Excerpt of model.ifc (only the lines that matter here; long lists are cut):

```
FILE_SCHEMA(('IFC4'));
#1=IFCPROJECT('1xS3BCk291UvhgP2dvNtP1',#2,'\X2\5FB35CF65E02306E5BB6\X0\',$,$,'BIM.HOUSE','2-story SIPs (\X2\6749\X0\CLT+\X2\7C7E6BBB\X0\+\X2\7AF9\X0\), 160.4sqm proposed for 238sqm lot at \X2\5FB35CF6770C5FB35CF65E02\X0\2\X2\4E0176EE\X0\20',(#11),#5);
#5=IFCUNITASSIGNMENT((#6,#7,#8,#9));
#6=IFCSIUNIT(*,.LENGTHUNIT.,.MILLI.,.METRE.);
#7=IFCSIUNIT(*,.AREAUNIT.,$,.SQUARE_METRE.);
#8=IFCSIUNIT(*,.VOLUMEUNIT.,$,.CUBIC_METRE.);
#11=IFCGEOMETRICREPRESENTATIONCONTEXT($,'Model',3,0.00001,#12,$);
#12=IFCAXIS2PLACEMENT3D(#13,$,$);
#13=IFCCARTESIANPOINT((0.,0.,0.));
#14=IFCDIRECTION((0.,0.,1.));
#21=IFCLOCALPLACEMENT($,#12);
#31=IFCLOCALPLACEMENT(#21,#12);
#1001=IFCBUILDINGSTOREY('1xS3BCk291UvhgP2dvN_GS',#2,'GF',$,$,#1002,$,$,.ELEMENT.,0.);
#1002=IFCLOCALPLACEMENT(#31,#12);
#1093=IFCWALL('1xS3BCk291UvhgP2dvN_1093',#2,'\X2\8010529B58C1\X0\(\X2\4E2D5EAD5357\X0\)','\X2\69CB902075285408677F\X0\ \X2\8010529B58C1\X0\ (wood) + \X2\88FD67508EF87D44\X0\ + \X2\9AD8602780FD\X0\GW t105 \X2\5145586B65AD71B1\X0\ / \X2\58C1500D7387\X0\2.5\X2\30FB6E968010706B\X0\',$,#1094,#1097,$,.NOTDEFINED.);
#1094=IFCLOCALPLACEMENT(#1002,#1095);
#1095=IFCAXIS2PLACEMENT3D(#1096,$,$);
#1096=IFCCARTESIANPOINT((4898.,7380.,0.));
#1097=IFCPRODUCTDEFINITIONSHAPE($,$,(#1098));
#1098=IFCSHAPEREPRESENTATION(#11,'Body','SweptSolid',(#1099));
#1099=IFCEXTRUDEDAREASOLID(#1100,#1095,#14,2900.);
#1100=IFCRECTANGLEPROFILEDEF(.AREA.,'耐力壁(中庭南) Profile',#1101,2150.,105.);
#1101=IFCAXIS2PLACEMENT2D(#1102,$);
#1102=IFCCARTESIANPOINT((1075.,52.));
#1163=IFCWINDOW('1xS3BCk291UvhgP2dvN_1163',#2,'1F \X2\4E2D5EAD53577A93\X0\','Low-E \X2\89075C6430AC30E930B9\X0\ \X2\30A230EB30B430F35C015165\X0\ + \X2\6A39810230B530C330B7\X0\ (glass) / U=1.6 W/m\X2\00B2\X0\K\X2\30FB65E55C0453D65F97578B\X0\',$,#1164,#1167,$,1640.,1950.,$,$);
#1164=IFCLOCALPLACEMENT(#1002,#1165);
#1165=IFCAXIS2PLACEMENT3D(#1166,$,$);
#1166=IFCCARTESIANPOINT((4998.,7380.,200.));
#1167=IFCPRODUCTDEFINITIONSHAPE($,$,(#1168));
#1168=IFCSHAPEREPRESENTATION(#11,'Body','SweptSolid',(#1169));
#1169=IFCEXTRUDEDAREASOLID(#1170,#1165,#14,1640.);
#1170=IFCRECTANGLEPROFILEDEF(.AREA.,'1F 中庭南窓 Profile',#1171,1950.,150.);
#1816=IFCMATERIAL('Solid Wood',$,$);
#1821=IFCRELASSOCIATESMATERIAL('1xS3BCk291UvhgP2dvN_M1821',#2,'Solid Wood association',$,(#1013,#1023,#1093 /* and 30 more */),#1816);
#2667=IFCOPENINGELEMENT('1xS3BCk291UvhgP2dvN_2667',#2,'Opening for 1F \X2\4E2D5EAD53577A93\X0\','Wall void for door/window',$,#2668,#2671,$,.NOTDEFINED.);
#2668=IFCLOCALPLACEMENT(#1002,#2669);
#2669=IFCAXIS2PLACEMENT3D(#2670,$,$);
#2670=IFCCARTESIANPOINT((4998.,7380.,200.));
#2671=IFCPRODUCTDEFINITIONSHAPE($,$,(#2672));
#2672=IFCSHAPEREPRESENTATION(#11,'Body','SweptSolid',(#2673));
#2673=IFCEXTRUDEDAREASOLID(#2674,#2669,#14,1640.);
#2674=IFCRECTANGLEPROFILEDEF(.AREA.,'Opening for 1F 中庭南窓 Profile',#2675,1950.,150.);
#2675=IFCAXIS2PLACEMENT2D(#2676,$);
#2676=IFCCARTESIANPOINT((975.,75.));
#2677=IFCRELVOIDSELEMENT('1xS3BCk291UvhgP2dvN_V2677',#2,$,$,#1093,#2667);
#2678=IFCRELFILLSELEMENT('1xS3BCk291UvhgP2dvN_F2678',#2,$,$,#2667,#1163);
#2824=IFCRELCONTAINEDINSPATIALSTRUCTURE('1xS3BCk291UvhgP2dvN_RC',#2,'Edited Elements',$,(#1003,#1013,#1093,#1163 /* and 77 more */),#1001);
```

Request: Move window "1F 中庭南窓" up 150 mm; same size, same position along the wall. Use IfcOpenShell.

```python
import numpy as np
import ifcopenshell
import ifcopenshell.api.geometry
import ifcopenshell.util.placement
import ifcopenshell.util.unit

model = ifcopenshell.open("model.ifc")
unit_scale = ifcopenshell.util.unit.calculate_unit_scale(model)

window = model.by_guid("1xS3BCk291UvhgP2dvN_1163")
opening = window.FillsVoids[0].RelatingOpeningElement
dz = 0.15 / unit_scale

shift = np.array([0.0, 0.0, dz])
# The window is not placed relative to its opening, so move both.
for product in (opening, window):
    matrix = ifcopenshell.util.placement.get_local_placement(product.ObjectPlacement)
    matrix[:3, 3] += shift
    ifcopenshell.api.geometry.edit_object_placement(model, product=product, matrix=matrix, is_si=False)

print(f"moved by {dz * unit_scale:+.3f} m")

model.write("model_v2.ifc")
```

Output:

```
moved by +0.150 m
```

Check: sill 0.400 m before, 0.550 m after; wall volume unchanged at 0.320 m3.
